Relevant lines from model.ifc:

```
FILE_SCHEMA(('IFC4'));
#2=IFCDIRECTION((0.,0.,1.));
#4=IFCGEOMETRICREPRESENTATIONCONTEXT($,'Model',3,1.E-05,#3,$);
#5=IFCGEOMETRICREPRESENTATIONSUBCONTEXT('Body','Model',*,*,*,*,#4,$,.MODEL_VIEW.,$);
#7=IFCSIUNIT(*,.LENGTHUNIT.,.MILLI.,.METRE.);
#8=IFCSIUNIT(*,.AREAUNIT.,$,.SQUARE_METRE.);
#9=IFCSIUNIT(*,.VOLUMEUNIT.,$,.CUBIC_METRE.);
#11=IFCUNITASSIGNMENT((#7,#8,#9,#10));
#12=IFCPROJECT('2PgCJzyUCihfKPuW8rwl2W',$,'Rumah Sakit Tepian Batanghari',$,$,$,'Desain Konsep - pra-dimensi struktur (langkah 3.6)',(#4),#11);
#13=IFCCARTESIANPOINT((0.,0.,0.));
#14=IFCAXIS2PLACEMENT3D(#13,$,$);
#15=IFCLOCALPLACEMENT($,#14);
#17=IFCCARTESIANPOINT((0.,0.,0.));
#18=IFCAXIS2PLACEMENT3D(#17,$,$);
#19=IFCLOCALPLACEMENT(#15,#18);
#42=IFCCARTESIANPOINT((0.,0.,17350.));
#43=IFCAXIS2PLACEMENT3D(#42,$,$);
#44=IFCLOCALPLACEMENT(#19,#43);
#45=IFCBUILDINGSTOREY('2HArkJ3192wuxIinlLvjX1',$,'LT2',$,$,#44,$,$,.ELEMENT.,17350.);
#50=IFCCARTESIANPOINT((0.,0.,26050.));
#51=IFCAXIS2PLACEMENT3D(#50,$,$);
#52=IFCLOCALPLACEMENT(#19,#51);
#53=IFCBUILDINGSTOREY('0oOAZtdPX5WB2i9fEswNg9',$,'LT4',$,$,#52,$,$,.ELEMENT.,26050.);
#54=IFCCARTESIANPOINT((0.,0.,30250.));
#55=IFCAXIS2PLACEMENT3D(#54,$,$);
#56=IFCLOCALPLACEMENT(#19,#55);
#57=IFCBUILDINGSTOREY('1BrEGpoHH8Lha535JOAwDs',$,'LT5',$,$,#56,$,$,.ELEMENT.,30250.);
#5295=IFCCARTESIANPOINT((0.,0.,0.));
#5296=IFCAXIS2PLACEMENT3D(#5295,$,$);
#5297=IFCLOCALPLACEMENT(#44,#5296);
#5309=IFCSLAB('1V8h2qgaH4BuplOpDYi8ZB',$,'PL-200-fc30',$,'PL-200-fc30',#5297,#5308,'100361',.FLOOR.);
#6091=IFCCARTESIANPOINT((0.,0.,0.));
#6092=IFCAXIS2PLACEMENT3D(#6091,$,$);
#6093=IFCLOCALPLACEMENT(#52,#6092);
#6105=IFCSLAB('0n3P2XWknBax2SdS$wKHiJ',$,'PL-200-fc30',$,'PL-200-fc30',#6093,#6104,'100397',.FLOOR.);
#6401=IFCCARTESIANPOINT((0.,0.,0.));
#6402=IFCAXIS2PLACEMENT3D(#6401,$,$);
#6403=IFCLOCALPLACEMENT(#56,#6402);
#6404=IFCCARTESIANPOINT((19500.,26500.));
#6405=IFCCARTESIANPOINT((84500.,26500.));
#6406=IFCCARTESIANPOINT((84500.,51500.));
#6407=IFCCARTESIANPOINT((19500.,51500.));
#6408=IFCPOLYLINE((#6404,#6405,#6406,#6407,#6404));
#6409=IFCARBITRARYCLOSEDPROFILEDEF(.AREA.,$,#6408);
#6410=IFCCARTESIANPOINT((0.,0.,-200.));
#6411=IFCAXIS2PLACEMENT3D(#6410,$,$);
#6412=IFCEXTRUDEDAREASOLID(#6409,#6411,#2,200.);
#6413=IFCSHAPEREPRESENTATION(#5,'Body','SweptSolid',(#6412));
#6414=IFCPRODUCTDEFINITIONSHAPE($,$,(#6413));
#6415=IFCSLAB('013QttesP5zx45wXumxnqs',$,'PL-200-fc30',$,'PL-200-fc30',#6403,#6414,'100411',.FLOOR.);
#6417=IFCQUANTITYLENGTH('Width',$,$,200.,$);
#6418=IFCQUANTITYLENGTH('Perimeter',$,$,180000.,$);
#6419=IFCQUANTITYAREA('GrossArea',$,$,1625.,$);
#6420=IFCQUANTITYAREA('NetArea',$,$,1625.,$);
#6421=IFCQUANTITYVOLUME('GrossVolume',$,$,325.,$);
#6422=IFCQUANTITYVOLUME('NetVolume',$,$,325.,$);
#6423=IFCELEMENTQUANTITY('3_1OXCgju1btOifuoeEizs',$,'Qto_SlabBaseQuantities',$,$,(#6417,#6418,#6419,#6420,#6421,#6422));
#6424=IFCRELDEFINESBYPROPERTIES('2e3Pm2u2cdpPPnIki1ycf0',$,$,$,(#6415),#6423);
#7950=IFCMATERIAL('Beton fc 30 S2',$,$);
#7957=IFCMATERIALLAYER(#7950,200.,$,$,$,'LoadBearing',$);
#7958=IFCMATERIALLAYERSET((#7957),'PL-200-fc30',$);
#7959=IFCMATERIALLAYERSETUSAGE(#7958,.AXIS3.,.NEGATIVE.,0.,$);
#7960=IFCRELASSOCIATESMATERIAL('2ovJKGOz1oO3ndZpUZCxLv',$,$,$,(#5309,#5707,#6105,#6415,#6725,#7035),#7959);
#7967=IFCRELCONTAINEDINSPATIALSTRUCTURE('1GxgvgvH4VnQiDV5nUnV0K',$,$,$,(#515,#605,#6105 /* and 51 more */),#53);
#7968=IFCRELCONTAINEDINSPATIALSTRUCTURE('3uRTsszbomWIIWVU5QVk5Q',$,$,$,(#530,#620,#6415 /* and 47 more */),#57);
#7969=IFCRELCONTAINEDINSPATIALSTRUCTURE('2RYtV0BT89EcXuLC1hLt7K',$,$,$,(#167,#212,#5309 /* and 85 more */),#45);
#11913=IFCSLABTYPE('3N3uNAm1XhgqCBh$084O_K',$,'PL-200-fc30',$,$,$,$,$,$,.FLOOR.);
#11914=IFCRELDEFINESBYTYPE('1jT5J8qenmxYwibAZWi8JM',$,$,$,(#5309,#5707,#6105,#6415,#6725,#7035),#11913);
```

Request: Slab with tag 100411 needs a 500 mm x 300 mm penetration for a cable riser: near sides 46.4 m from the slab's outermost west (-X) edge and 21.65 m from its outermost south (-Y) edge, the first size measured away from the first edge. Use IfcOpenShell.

```python
import numpy as np
import ifcopenshell
import ifcopenshell.api.feature
import ifcopenshell.api.geometry
import ifcopenshell.api.pset
import ifcopenshell.api.root
import ifcopenshell.geom
import ifcopenshell.util.element
import ifcopenshell.util.placement
import ifcopenshell.util.representation
import ifcopenshell.util.shape
import ifcopenshell.util.unit

model = ifcopenshell.open("model.ifc")
unit_scale = ifcopenshell.util.unit.calculate_unit_scale(model)
area_scale = ifcopenshell.util.unit.calculate_unit_scale(model, "AREAUNIT")
volume_scale = ifcopenshell.util.unit.calculate_unit_scale(model, "VOLUMEUNIT")
settings = ifcopenshell.geom.settings()


def volume(element):
    """Net volume in cubic metres, openings subtracted."""
    shape = ifcopenshell.geom.create_shape(settings, element)
    return ifcopenshell.util.shape.get_volume(shape.geometry)


slab = model.by_guid("013QttesP5zx45wXumxnqs")
before = volume(slab)

# Extent in the slab's own axes, in metres. The edges named are its -X and -Y sides.
slab_shape = ifcopenshell.geom.create_shape(settings, slab)
vertices = ifcopenshell.util.shape.get_vertices(slab_shape.geometry)
x_min, y_min, bottom = vertices.min(axis=0)
top = vertices[:, 2].max()

opening = ifcopenshell.api.root.create_entity(model, ifc_class="IfcOpeningElement", name="Cable riser opening", predefined_type="OPENING")
context = ifcopenshell.util.representation.get_context(model, "Model", "Body", "MODEL_VIEW")
width, depth = 0.5, 0.3
outline = [(0.0, 0.0), (width, 0.0), (width, depth), (0.0, depth), (0.0, 0.0)]
# Overshoot both faces by 50 mm so the cut is clean.
shape = ifcopenshell.api.geometry.add_slab_representation(
    model, context=context, depth=top - bottom + 0.1, polyline=outline
)
ifcopenshell.api.geometry.assign_representation(model, product=opening, representation=shape)

matrix = ifcopenshell.util.placement.get_local_placement(slab.ObjectPlacement)
matrix[:, 3] = matrix @ np.append(np.array([x_min + 46.4, y_min + 21.65, bottom - 0.05]) / unit_scale, 1.0)
ifcopenshell.api.geometry.edit_object_placement(model, product=opening, matrix=matrix, is_si=False)
ifcopenshell.api.feature.add_feature(model, feature=opening, element=slab)

after = volume(slab)

# Update the slab's stored quantities.
qto = model.by_id(ifcopenshell.util.element.get_pset(slab, "Qto_SlabBaseQuantities", should_inherit=False)["id"])
ifcopenshell.api.pset.edit_qto(model, qto=qto, properties={
    "NetArea": after / (top - bottom) / area_scale,
    "NetVolume": after / volume_scale,
})

print(f"slab volume {before:.3f} -> {after:.3f} m3")

model.write("model_rev.ifc")
```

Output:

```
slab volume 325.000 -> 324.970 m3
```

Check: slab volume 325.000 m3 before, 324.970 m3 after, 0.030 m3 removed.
